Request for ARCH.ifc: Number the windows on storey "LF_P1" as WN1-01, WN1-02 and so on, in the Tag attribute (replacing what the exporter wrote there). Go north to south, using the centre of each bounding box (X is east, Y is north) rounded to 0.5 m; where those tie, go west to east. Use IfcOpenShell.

First a look at what the model holds.

```python
import ifcopenshell
import ifcopenshell.util.element
import ifcopenshell.util.placement

model = ifcopenshell.open("ARCH.ifc")
print(model.schema)
storey = next(s for s in model.by_type("IfcBuildingStorey") if s.Name == "LF_P1")
windows = [e for e in ifcopenshell.util.element.get_decomposition(storey) if e.is_a("IfcWindow")]
for e in sorted(windows, key=lambda e: e.id()):
    origin = ifcopenshell.util.placement.get_local_placement(e.ObjectPlacement)[:3, 3]
    print(e.id(), e.Tag, e.Name, origin.round(2) + 0.0, sep=" | ")
```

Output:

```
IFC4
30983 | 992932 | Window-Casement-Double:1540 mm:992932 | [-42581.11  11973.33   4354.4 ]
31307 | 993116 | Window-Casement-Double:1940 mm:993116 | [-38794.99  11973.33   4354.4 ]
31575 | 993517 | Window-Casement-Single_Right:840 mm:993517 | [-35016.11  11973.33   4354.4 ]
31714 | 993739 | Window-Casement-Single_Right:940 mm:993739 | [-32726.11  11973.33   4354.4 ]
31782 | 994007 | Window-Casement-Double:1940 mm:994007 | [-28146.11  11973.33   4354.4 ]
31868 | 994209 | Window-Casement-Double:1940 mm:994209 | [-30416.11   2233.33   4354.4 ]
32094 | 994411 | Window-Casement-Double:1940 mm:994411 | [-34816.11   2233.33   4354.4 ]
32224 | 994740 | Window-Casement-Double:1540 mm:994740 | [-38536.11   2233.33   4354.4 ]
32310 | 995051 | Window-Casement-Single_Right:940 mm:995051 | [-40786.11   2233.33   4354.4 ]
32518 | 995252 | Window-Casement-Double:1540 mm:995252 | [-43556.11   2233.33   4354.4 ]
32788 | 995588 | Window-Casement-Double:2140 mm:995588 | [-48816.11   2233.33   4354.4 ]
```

```python
import ifcopenshell
import ifcopenshell.geom
import ifcopenshell.util.element
import ifcopenshell.util.shape

model = ifcopenshell.open("ARCH.ifc")
settings = ifcopenshell.geom.settings()
settings.set("use-world-coords", True)


def centre(element):
    shape = ifcopenshell.geom.create_shape(settings, element)
    return ifcopenshell.util.shape.get_bbox_centroid(shape.geometry)


storey = next(s for s in model.by_type("IfcBuildingStorey") if s.Name == "LF_P1")
windows = [e for e in ifcopenshell.util.element.get_decomposition(storey) if e.is_a("IfcWindow")]

# Insertion points can sit at a corner or the storey origin, so sort by the geometry (in metres).
centres = {e: centre(e) for e in windows}
windows.sort(key=lambda e: (-round(centres[e][1] / 0.5), centres[e][0]))

for i, e in enumerate(windows, start=1):
    number = f"WN1-{i:02d}"
    e.Tag = number
    print(e.id(), number)

model.write("ARCH_updated.ifc")
```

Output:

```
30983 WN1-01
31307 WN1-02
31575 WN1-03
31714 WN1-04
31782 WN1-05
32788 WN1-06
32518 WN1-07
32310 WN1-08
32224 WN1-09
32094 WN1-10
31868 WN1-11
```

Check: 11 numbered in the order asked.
